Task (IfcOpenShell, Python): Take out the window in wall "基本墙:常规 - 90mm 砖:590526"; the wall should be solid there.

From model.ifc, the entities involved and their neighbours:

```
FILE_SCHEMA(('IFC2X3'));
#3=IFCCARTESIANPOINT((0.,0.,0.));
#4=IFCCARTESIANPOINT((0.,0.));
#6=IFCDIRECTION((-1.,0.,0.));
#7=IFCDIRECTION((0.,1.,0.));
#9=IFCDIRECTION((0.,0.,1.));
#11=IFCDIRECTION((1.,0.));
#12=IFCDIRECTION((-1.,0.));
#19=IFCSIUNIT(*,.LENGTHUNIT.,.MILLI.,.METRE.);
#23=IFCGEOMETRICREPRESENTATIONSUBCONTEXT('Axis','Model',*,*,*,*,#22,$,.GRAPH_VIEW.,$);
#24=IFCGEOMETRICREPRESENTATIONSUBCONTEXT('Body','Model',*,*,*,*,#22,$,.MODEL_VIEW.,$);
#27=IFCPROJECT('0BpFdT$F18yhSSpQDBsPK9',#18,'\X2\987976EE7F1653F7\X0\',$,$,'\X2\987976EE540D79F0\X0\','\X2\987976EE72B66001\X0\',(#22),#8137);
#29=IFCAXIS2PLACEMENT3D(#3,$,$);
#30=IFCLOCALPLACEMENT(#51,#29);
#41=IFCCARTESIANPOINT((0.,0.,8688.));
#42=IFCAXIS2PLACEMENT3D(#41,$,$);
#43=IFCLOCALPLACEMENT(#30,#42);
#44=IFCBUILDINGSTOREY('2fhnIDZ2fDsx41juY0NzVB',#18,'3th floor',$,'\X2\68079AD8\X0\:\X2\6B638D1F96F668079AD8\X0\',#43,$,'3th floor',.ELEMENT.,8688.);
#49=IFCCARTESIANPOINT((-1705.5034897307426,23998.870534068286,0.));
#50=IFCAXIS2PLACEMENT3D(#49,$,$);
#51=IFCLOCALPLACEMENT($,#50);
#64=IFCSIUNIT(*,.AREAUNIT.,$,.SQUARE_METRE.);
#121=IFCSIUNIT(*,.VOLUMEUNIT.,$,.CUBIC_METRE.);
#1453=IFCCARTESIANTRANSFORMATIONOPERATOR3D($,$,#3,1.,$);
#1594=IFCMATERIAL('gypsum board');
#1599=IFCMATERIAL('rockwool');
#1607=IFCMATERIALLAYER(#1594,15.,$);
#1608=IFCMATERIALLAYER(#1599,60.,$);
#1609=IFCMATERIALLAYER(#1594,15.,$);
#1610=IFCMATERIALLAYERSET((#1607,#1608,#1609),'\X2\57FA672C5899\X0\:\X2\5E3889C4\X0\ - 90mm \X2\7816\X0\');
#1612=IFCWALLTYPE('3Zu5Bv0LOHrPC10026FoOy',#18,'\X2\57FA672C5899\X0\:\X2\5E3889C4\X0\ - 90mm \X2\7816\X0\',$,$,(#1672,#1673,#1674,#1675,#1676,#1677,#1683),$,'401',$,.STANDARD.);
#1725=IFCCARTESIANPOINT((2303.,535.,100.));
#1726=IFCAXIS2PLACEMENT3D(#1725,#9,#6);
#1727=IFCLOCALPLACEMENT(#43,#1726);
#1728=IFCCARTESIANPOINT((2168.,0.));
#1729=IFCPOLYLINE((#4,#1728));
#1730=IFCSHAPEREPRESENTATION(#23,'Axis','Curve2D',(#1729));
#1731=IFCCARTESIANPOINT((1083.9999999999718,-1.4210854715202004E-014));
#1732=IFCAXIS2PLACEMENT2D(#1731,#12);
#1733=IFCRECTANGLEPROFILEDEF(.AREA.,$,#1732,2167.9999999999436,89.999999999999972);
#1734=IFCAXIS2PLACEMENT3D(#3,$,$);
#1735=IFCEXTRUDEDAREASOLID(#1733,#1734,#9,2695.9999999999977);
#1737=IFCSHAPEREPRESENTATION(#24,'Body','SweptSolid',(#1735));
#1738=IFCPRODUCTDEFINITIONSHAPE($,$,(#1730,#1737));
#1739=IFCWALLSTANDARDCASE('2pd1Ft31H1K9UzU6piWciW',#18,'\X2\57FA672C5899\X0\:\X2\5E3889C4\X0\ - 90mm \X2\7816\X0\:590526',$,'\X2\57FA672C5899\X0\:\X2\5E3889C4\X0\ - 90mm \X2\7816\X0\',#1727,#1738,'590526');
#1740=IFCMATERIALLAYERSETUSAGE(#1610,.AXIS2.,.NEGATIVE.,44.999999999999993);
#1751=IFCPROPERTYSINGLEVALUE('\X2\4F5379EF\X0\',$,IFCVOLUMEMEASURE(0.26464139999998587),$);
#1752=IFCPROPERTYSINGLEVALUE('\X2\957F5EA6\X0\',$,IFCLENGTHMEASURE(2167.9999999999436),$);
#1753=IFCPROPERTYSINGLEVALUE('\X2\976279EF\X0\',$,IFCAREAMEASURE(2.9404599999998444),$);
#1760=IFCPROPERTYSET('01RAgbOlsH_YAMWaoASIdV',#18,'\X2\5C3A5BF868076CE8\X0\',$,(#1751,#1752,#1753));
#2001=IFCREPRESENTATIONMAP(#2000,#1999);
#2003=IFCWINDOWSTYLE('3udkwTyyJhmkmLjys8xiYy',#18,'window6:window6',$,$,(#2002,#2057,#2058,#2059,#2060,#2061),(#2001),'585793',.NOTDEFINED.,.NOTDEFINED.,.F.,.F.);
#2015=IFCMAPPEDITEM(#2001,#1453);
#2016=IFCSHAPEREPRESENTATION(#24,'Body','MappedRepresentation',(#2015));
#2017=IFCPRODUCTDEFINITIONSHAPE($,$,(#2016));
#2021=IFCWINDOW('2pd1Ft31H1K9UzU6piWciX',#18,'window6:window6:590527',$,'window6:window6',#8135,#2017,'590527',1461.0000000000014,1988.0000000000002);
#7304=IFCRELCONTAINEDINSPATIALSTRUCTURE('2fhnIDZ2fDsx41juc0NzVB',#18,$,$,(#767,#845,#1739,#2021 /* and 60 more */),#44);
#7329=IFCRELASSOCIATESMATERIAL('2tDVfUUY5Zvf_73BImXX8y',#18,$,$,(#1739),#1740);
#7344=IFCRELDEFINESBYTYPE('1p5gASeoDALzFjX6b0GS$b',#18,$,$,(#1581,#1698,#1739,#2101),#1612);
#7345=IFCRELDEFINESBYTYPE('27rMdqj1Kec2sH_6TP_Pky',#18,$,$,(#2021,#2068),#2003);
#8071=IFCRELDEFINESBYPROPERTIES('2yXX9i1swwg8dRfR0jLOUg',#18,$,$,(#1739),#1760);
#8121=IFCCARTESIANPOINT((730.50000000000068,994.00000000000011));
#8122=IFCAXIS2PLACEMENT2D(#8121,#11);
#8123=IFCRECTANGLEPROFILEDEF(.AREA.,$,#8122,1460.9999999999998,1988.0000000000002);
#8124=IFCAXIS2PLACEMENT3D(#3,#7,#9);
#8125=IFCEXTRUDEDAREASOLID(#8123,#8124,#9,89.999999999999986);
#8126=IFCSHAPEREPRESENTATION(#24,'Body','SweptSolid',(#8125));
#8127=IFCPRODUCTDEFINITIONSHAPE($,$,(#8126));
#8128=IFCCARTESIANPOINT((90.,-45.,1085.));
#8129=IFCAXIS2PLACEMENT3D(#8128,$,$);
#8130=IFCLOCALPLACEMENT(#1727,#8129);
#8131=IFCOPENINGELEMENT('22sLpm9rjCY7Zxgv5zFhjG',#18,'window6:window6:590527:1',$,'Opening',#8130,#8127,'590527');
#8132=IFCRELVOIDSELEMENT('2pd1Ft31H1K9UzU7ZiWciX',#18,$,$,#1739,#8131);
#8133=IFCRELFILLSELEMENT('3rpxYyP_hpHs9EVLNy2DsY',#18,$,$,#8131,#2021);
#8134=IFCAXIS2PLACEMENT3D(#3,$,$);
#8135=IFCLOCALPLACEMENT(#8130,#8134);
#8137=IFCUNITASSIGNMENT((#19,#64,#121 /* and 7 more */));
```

```python
import ifcopenshell
import ifcopenshell.api.feature
import ifcopenshell.api.pset
import ifcopenshell.api.root
import ifcopenshell.geom
import ifcopenshell.util.element
import ifcopenshell.util.shape
import ifcopenshell.util.unit

model = ifcopenshell.open("model.ifc")
area_scale = ifcopenshell.util.unit.calculate_unit_scale(model, "AREAUNIT")
volume_scale = ifcopenshell.util.unit.calculate_unit_scale(model, "VOLUMEUNIT")
settings = ifcopenshell.geom.settings()


def volume(element):
    """Net volume in cubic metres, openings subtracted."""
    shape = ifcopenshell.geom.create_shape(settings, element)
    return ifcopenshell.util.shape.get_volume(shape.geometry)


window = model.by_id(2021)
opening = window.FillsVoids[0].RelatingOpeningElement
wall = opening.VoidsElements[0].RelatingBuildingElement
before = volume(wall)

ifcopenshell.api.root.remove_product(model, product=window)
ifcopenshell.api.feature.remove_feature(model, feature=opening)

after = volume(wall)
thickness = 0.09  # wall thickness in metres

# Update the wall's stored quantities.
pset = model.by_id(ifcopenshell.util.element.get_pset(wall, "尺寸标注", should_inherit=False)["id"])
ifcopenshell.api.pset.edit_pset(model, pset=pset, properties={
    "体积": model.create_entity("IfcVolumeMeasure", after / volume_scale),
    "面积": model.create_entity("IfcAreaMeasure", after / thickness / area_scale),
})

print(f"wall volume {before:.3f} -> {after:.3f} m3")

model.write("model_v2.ifc")
```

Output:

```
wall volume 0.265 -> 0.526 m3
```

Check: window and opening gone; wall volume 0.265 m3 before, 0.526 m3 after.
